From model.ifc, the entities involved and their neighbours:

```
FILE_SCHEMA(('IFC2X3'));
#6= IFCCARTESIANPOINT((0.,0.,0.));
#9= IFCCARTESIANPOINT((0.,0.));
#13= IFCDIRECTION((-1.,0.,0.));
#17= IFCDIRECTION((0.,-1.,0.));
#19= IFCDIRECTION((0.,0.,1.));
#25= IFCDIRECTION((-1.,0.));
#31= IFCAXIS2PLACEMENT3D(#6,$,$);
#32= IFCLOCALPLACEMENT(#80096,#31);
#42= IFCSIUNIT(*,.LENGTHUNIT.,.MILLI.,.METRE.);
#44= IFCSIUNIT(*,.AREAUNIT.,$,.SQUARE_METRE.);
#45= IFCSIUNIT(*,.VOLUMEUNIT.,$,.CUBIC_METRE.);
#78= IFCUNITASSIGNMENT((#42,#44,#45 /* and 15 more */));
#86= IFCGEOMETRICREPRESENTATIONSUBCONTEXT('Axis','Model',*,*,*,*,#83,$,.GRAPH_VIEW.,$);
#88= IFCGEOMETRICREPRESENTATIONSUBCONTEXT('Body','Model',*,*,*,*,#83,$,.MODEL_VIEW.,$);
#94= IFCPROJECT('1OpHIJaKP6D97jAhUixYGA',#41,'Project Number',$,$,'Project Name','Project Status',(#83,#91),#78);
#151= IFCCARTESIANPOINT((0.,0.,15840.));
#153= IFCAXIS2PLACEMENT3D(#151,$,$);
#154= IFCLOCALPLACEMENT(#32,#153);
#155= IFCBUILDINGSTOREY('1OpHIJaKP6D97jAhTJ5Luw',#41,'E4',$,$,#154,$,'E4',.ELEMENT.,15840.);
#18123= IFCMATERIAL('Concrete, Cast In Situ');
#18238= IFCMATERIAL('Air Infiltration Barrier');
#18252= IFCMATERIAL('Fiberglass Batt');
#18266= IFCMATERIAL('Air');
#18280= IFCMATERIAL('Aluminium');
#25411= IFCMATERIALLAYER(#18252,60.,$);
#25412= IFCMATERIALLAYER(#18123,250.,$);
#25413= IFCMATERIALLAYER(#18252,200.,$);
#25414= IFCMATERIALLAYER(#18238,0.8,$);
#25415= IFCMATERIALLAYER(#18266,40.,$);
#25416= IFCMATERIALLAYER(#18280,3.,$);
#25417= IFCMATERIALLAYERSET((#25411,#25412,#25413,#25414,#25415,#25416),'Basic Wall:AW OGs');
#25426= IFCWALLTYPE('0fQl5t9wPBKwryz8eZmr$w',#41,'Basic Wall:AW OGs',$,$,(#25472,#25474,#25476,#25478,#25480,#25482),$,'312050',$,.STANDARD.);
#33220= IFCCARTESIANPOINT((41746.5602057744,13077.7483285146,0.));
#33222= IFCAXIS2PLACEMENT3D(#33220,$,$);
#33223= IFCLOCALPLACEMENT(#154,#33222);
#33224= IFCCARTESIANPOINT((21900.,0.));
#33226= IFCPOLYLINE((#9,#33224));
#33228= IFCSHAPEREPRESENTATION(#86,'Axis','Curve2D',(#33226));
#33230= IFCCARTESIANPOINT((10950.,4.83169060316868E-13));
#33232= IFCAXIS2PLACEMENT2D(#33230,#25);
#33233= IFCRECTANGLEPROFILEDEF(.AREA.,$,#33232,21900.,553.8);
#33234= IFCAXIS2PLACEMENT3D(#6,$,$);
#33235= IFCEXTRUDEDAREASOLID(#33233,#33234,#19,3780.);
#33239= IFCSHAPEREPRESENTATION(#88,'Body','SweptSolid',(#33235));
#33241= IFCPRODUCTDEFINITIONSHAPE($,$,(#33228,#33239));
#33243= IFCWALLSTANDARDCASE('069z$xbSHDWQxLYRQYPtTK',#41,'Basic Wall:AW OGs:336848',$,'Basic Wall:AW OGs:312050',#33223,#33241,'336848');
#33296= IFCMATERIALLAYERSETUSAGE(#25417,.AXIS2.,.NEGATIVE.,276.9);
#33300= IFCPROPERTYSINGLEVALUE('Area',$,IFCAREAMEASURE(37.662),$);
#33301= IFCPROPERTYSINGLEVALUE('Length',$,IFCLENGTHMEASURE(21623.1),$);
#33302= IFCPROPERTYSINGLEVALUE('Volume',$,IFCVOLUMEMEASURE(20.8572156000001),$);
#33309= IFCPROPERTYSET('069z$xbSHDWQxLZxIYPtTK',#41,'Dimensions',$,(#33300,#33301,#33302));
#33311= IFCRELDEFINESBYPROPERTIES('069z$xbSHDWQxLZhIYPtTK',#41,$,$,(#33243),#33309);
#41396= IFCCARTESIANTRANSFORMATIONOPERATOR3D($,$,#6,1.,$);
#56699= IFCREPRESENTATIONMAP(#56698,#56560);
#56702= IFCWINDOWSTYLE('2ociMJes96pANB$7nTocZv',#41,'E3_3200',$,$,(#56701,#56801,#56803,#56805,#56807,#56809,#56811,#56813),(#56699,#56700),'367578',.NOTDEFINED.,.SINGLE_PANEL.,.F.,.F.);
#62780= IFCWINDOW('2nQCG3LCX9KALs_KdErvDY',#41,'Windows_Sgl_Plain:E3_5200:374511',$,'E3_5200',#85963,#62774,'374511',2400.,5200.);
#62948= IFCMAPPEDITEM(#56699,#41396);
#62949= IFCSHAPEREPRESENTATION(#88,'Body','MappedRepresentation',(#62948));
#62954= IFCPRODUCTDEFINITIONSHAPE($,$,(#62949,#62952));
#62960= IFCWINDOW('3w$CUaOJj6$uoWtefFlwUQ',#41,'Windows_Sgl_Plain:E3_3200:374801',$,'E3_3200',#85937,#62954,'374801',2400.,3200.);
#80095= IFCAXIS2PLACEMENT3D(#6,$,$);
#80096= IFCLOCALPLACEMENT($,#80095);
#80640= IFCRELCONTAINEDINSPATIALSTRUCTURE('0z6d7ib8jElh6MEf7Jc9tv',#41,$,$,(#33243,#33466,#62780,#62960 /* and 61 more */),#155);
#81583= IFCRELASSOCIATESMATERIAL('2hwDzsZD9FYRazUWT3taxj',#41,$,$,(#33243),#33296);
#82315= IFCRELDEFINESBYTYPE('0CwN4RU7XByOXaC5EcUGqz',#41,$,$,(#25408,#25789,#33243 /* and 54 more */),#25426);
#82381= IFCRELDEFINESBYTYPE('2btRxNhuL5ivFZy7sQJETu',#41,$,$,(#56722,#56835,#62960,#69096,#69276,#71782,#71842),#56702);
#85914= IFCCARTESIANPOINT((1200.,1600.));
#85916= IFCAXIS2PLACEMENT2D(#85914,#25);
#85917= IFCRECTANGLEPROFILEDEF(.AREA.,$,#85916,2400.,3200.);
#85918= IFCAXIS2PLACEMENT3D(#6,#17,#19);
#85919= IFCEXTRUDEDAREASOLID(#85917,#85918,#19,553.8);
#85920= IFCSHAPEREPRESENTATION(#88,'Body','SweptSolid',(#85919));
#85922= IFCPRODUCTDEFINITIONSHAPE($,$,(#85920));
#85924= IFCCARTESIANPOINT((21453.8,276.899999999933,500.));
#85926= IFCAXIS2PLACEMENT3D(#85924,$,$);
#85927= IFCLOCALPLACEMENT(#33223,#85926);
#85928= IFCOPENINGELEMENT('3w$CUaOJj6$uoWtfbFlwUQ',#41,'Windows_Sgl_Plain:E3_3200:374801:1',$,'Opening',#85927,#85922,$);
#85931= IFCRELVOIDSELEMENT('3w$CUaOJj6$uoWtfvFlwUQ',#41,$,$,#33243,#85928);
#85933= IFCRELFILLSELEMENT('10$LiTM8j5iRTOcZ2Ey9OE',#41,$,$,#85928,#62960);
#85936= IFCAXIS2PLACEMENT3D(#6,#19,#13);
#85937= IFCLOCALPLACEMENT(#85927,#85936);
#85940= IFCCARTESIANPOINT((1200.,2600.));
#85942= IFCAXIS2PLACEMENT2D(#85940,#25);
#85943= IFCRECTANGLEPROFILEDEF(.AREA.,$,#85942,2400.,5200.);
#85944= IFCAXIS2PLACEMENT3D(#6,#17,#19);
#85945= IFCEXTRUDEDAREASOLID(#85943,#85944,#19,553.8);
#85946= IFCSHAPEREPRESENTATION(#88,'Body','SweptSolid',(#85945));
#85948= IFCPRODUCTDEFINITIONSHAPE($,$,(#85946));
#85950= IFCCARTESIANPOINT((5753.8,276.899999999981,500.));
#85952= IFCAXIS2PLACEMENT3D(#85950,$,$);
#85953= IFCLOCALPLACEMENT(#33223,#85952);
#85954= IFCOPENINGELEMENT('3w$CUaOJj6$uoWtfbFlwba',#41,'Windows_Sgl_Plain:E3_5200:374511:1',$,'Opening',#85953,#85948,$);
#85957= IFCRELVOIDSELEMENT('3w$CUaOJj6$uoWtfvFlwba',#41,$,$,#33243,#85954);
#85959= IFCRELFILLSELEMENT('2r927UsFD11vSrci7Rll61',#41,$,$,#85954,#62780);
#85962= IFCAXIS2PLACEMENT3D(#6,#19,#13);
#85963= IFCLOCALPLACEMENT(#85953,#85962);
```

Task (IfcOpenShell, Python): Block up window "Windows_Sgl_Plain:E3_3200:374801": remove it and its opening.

```python
import ifcopenshell
import ifcopenshell.api.feature
import ifcopenshell.api.pset
import ifcopenshell.api.root
import ifcopenshell.geom
import ifcopenshell.util.element
import ifcopenshell.util.shape
import ifcopenshell.util.unit

model = ifcopenshell.open("model.ifc")
area_scale = ifcopenshell.util.unit.calculate_unit_scale(model, "AREAUNIT")
volume_scale = ifcopenshell.util.unit.calculate_unit_scale(model, "VOLUMEUNIT")
settings = ifcopenshell.geom.settings()


def volume(element):
    """Net volume in cubic metres, openings subtracted."""
    shape = ifcopenshell.geom.create_shape(settings, element)
    return ifcopenshell.util.shape.get_volume(shape.geometry)


window = model.by_guid("3w$CUaOJj6$uoWtefFlwUQ")
opening = window.FillsVoids[0].RelatingOpeningElement
wall = opening.VoidsElements[0].RelatingBuildingElement
before = volume(wall)

ifcopenshell.api.root.remove_product(model, product=window)
ifcopenshell.api.feature.remove_feature(model, feature=opening)

after = volume(wall)
thickness = 0.5538  # wall thickness in metres

# Update the wall's stored quantities.
pset = model.by_id(ifcopenshell.util.element.get_pset(wall, "Dimensions", should_inherit=False)["id"])
ifcopenshell.api.pset.edit_pset(model, pset=pset, properties={
    "Area": model.create_entity("IfcAreaMeasure", after / thickness / area_scale),
    "Volume": model.create_entity("IfcVolumeMeasure", after / volume_scale),
})

print(f"wall volume {before:.3f} -> {after:.3f} m3")

model.write("model_rev.ifc")
```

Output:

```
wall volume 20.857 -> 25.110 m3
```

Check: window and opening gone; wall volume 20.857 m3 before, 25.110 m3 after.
